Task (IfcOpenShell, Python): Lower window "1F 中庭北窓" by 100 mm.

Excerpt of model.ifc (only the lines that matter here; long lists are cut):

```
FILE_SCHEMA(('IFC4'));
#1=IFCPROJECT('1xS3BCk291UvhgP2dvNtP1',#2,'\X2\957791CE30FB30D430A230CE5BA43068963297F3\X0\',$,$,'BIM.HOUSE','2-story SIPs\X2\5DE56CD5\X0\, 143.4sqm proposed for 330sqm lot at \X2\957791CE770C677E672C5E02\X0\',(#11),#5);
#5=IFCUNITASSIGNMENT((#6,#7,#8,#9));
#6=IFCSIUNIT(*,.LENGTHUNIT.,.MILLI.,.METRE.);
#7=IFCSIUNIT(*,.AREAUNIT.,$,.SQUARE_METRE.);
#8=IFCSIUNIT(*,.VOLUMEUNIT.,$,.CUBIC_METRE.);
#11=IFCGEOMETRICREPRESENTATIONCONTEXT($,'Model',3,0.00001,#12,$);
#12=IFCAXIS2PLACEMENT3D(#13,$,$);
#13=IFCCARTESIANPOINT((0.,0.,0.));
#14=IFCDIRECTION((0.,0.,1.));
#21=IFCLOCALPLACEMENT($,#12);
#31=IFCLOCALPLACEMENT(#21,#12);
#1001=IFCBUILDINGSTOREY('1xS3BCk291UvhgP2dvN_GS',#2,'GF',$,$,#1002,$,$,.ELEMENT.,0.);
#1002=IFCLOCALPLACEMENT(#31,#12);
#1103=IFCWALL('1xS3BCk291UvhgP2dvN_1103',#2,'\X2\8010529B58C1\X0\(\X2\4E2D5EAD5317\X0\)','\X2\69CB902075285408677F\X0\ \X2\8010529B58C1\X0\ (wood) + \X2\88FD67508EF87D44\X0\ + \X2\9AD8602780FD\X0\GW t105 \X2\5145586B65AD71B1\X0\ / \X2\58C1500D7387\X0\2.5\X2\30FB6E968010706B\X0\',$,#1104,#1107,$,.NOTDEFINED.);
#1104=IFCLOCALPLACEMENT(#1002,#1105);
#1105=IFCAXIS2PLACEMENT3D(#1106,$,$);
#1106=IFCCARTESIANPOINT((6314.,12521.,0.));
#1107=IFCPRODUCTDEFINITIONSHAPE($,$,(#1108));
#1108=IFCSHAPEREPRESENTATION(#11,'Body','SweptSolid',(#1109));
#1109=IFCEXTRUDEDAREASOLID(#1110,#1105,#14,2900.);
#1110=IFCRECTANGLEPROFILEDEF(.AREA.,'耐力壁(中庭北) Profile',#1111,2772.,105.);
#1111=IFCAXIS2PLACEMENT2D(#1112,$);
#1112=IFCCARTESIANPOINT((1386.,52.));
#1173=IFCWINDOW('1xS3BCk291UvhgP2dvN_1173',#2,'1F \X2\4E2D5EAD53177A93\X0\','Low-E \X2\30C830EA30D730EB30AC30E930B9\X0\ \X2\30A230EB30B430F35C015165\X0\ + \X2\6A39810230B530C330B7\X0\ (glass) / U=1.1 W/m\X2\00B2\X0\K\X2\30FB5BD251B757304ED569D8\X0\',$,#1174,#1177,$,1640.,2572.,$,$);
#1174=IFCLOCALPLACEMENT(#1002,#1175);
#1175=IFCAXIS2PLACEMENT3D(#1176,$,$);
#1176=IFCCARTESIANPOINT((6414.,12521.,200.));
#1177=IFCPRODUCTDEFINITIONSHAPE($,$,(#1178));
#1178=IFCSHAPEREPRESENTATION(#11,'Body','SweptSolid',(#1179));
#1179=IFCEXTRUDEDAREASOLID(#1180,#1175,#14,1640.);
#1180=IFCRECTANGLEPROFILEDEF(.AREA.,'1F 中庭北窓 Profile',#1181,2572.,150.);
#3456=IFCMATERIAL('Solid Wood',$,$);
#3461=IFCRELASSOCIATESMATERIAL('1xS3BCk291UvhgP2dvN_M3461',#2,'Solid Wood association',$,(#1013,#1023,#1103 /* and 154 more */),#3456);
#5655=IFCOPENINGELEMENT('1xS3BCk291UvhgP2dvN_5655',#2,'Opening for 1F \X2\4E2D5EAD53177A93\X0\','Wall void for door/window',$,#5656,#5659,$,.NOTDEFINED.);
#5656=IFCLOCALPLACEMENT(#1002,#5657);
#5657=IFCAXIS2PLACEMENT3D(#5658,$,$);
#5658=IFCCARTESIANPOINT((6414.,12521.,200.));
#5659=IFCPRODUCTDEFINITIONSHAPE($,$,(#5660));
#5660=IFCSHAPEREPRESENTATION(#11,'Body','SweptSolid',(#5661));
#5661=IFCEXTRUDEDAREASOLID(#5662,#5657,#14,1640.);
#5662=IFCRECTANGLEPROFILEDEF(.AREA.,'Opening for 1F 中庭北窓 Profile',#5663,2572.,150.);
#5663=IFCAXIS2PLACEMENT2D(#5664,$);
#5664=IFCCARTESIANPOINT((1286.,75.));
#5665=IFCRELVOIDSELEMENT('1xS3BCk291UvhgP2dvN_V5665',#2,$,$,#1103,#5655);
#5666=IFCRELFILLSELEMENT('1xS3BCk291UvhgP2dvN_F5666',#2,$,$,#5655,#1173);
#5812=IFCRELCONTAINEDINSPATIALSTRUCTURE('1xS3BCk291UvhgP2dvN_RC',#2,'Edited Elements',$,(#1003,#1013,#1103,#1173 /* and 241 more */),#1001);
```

```python
import numpy as np
import ifcopenshell
import ifcopenshell.api.geometry
import ifcopenshell.util.placement
import ifcopenshell.util.unit

model = ifcopenshell.open("model.ifc")
unit_scale = ifcopenshell.util.unit.calculate_unit_scale(model)

window = model.by_guid("1xS3BCk291UvhgP2dvN_1173")
opening = window.FillsVoids[0].RelatingOpeningElement
dz = -0.1 / unit_scale

shift = np.array([0.0, 0.0, dz])
# The window is not placed relative to its opening, so move both.
for product in (opening, window):
    matrix = ifcopenshell.util.placement.get_local_placement(product.ObjectPlacement)
    matrix[:3, 3] += shift
    ifcopenshell.api.geometry.edit_object_placement(model, product=product, matrix=matrix, is_si=False)

print(f"moved by {dz * unit_scale:+.3f} m")

model.write("model_v2.ifc")
```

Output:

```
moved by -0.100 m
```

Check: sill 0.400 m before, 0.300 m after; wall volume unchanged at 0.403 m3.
